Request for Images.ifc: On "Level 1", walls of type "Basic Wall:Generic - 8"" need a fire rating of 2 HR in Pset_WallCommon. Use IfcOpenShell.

First a look at what the model holds.

```python
import ifcopenshell
import ifcopenshell.util.element

model = ifcopenshell.open("Images.ifc")
print(model.schema)
storey = next(s for s in model.by_type("IfcBuildingStorey") if s.Name == "Level 1")
walls = [e for e in ifcopenshell.util.element.get_decomposition(storey) if e.is_a("IfcWall")]
seen = {}
for e in walls:
    element_type = ifcopenshell.util.element.get_type(e)
    key = (element_type.Name if element_type != e and element_type else None, ifcopenshell.util.element.get_pset(e, "Pset_WallCommon", "FireRating"))
    seen[key] = seen.get(key, 0) + 1
for (name, value), count in sorted(seen.items(), key=str):
    print(count, "x", name, "|", value)
```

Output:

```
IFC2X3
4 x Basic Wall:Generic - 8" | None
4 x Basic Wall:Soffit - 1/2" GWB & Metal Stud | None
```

```python
import ifcopenshell
import ifcopenshell.api.pset
import ifcopenshell.util.element

model = ifcopenshell.open("Images.ifc")

storey = next(s for s in model.by_type("IfcBuildingStorey") if s.Name == "Level 1")
walls = [e for e in ifcopenshell.util.element.get_decomposition(storey) if e.is_a("IfcWall")]

count = 0
for e in walls:
    element_type = ifcopenshell.util.element.get_type(e)
    if element_type in (None, e) or element_type.Name != 'Basic Wall:Generic - 8"':
        continue
    # add_pset returns the element's existing set when there is one.
    pset = ifcopenshell.api.pset.add_pset(model, product=e, name="Pset_WallCommon")
    ifcopenshell.api.pset.edit_pset(model, pset=pset, properties={"FireRating": "2 HR"})
    count += 1

print(count, "walls updated")

model.write("Images_updated.ifc")
```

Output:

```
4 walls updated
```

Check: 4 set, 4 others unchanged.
